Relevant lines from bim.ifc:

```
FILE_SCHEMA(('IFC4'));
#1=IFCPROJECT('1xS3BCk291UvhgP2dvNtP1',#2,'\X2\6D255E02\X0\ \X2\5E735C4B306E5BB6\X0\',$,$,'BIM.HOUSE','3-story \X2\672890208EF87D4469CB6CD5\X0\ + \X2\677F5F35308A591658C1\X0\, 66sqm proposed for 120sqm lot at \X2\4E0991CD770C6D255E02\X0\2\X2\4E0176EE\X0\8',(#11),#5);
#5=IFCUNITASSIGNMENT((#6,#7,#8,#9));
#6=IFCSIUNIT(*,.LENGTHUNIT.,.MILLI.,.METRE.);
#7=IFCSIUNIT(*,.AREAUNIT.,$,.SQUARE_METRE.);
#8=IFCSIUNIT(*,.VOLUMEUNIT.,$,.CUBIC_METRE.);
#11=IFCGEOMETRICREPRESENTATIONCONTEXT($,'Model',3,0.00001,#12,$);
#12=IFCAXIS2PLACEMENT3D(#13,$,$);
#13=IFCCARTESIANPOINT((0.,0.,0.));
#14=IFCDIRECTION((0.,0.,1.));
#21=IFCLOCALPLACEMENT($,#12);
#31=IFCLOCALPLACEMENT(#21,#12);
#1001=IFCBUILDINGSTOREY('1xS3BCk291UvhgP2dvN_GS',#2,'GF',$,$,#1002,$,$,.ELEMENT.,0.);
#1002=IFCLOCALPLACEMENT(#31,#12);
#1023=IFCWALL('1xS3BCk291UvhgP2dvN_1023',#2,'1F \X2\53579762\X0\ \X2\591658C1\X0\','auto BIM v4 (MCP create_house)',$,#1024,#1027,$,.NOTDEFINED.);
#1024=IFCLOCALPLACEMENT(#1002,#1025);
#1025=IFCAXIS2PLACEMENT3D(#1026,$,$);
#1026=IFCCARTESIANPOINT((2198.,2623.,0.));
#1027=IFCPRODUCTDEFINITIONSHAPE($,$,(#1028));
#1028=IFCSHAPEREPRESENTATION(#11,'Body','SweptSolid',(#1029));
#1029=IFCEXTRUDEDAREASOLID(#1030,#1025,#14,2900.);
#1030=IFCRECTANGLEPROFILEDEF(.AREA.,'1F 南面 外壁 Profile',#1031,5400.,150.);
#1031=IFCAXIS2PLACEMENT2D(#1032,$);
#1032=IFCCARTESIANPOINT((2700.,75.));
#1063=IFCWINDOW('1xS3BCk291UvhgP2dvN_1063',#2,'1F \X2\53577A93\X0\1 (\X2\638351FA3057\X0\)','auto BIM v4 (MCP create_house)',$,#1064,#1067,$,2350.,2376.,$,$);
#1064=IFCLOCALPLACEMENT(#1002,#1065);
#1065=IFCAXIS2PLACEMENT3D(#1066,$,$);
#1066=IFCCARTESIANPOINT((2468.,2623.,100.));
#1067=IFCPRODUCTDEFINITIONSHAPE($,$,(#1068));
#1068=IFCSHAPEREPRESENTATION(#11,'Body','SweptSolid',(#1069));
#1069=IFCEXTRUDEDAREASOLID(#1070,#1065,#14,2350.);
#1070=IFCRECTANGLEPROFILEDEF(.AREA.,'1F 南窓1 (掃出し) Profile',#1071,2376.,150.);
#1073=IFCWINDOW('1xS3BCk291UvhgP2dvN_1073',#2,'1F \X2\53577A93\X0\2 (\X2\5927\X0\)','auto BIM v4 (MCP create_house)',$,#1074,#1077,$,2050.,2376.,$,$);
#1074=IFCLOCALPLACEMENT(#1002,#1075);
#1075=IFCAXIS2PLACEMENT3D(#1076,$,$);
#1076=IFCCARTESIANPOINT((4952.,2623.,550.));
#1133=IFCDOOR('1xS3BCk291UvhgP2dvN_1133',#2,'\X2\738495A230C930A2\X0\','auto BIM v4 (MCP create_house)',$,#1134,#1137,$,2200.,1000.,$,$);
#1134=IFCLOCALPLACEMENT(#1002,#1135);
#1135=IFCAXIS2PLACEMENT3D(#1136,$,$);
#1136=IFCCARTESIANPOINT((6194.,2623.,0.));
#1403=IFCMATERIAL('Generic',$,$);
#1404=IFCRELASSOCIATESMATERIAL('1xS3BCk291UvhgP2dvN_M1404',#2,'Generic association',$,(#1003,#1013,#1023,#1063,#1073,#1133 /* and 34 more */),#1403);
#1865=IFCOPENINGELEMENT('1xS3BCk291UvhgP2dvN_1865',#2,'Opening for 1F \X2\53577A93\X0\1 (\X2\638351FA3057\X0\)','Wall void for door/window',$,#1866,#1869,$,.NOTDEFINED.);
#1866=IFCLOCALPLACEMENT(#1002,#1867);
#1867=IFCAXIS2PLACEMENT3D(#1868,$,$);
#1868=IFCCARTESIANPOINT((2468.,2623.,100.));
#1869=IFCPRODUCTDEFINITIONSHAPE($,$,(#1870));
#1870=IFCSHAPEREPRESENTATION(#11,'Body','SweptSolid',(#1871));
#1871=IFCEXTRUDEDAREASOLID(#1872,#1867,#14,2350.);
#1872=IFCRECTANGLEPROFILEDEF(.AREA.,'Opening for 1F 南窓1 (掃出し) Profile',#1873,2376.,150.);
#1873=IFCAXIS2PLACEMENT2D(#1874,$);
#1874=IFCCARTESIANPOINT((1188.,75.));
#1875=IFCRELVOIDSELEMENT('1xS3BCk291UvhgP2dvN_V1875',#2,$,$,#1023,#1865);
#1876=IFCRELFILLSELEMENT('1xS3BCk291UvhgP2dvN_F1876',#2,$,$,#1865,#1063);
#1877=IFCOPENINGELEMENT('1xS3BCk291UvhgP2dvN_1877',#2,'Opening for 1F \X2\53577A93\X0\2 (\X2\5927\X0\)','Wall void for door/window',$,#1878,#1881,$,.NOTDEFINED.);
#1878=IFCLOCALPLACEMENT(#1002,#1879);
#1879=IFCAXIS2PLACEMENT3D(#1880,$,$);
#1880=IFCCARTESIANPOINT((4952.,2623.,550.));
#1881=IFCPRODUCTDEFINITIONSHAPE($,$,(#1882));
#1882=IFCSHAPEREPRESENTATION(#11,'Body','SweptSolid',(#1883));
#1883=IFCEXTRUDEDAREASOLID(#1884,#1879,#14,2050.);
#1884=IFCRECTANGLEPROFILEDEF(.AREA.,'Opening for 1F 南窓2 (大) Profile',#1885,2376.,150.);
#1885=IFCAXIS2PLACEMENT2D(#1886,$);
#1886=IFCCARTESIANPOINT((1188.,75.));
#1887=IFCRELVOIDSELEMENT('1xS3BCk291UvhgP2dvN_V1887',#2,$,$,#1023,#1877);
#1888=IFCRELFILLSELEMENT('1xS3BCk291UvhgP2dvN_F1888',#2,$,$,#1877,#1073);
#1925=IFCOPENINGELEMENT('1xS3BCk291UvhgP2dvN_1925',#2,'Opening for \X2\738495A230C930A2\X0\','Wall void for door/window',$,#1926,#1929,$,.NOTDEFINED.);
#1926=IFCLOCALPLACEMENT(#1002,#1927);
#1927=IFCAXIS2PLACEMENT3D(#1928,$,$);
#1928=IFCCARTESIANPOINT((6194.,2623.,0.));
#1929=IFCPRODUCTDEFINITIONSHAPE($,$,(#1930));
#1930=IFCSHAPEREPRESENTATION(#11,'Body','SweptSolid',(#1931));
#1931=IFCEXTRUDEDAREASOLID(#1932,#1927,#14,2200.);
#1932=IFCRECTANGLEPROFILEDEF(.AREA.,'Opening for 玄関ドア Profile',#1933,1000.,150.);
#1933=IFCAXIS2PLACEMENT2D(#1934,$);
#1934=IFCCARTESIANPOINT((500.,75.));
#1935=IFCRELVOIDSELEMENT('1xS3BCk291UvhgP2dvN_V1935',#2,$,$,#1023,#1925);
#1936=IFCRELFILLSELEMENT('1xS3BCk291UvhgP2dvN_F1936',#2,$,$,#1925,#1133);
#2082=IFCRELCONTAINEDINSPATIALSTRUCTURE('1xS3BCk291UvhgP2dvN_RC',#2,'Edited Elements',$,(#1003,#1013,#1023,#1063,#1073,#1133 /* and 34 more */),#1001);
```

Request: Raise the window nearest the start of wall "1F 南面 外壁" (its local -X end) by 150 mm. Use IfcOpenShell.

```python
import numpy as np
import ifcopenshell
import ifcopenshell.api.geometry
import ifcopenshell.util.placement
import ifcopenshell.util.unit

model = ifcopenshell.open("bim.ifc")
unit_scale = ifcopenshell.util.unit.calculate_unit_scale(model)

window = model.by_guid("1xS3BCk291UvhgP2dvN_1063")
opening = window.FillsVoids[0].RelatingOpeningElement
dz = 150.0

shift = np.array([0.0, 0.0, dz])
# The window is not placed relative to its opening, so move both.
for product in (opening, window):
    matrix = ifcopenshell.util.placement.get_local_placement(product.ObjectPlacement)
    matrix[:3, 3] += shift
    ifcopenshell.api.geometry.edit_object_placement(model, product=product, matrix=matrix, is_si=False)

print(f"moved by {dz * unit_scale:+.3f} m")

model.write("bim_v2.ifc")
```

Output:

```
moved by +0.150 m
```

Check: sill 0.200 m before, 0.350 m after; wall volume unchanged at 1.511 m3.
